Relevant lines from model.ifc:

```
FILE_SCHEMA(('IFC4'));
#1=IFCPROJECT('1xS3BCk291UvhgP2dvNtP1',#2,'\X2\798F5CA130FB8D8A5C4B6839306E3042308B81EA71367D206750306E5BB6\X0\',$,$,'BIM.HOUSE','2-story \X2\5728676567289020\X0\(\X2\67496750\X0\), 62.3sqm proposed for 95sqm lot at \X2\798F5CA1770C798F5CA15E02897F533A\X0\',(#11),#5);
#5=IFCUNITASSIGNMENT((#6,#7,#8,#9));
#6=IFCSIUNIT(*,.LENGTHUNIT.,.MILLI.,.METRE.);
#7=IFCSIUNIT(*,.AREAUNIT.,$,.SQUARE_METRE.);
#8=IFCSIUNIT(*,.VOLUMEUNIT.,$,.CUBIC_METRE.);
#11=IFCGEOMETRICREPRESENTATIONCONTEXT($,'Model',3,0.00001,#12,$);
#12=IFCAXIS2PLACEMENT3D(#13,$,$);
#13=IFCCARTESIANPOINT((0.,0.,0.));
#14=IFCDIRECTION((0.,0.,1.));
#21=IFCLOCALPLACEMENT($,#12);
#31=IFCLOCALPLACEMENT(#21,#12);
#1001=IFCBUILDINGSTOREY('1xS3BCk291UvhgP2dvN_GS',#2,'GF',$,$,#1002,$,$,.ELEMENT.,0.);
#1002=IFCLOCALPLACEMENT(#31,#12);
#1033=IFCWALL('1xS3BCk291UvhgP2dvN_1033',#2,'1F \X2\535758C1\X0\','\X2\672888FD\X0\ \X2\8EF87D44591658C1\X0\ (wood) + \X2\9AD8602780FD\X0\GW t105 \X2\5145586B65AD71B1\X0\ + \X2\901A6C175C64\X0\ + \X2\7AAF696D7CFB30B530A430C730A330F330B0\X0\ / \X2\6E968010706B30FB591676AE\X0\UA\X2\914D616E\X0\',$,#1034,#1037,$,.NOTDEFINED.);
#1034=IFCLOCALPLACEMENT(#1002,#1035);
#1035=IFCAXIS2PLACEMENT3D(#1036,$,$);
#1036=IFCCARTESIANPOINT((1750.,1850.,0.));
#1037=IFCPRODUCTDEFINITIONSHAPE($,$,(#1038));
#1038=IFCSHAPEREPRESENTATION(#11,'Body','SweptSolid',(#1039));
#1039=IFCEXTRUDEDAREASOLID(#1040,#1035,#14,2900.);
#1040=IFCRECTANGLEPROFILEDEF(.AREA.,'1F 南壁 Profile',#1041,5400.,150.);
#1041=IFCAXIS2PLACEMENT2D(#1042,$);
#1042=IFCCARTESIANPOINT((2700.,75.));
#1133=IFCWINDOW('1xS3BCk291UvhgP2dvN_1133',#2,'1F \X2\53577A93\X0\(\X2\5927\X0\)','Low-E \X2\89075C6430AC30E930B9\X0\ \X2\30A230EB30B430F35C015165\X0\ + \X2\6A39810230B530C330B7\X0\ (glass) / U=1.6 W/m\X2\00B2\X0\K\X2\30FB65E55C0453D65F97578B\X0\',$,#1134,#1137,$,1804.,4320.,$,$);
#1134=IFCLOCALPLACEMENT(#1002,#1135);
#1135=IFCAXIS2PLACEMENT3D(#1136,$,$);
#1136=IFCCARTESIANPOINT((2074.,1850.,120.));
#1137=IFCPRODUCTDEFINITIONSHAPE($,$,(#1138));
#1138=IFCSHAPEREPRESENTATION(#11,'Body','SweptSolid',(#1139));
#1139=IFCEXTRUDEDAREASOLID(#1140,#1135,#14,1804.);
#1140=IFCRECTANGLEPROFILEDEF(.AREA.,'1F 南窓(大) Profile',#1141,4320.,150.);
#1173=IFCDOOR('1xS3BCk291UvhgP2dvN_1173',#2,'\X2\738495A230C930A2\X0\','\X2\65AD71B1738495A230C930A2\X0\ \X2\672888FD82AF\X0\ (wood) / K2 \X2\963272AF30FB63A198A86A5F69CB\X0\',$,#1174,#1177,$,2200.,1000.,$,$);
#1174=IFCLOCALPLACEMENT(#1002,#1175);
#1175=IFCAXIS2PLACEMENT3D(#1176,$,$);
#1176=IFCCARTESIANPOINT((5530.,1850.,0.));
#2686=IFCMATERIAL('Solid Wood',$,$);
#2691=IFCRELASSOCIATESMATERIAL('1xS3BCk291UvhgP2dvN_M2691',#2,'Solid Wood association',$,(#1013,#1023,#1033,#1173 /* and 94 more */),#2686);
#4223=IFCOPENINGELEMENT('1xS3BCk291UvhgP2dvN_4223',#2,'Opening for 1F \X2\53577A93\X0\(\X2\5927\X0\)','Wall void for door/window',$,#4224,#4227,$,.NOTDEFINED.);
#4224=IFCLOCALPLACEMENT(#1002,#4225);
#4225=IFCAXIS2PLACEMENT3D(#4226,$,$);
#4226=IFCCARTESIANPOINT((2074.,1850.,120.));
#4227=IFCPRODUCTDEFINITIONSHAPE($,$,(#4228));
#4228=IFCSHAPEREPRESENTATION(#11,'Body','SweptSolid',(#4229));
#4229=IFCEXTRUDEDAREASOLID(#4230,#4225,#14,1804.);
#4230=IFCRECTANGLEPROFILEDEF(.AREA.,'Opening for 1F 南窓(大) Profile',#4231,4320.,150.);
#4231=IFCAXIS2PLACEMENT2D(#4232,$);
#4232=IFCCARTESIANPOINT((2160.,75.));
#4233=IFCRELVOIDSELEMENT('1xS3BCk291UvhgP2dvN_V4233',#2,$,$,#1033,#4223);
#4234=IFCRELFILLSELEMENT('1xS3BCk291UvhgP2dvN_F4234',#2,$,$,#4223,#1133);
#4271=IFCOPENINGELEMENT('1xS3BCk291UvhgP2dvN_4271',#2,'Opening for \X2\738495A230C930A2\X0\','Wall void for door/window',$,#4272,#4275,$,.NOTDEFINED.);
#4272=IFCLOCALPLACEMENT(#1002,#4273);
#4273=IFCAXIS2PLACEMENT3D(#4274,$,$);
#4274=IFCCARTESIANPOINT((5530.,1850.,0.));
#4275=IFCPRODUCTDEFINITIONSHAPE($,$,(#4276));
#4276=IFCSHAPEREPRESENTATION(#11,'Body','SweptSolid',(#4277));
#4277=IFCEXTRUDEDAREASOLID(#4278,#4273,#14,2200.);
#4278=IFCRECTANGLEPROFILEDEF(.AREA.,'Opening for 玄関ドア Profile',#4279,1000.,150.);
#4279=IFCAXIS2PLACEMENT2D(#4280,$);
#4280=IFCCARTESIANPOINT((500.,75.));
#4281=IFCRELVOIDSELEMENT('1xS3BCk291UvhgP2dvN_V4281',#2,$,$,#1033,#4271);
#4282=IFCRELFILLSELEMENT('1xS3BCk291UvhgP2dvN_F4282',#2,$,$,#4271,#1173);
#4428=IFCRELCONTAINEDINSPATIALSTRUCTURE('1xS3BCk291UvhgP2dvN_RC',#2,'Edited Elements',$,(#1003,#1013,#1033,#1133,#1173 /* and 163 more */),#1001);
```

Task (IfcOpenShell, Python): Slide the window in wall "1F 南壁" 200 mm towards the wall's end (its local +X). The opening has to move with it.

```python
import ifcopenshell
import ifcopenshell.api.geometry
import ifcopenshell.util.placement
import ifcopenshell.util.unit

model = ifcopenshell.open("model.ifc")
unit_scale = ifcopenshell.util.unit.calculate_unit_scale(model)

window = model.by_id(1133)
opening = window.FillsVoids[0].RelatingOpeningElement
wall = opening.VoidsElements[0].RelatingBuildingElement

wall_matrix = ifcopenshell.util.placement.get_local_placement(wall.ObjectPlacement)
shift = wall_matrix[:3, 0] * 0.2 / unit_scale
before = ifcopenshell.util.placement.get_local_placement(window.ObjectPlacement)[:3, 3].copy()

# The window is not placed relative to its opening, so move both.
for product in (opening, window):
    matrix = ifcopenshell.util.placement.get_local_placement(product.ObjectPlacement)
    matrix[:3, 3] += shift
    ifcopenshell.api.geometry.edit_object_placement(model, product=product, matrix=matrix, is_si=False)

after = ifcopenshell.util.placement.get_local_placement(window.ObjectPlacement)[:3, 3]
print("window moved by", (after - before).round(3) + 0.0)

model.write("model_updated.ifc")
```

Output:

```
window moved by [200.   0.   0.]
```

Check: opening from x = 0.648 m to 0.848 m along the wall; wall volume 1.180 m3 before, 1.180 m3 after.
